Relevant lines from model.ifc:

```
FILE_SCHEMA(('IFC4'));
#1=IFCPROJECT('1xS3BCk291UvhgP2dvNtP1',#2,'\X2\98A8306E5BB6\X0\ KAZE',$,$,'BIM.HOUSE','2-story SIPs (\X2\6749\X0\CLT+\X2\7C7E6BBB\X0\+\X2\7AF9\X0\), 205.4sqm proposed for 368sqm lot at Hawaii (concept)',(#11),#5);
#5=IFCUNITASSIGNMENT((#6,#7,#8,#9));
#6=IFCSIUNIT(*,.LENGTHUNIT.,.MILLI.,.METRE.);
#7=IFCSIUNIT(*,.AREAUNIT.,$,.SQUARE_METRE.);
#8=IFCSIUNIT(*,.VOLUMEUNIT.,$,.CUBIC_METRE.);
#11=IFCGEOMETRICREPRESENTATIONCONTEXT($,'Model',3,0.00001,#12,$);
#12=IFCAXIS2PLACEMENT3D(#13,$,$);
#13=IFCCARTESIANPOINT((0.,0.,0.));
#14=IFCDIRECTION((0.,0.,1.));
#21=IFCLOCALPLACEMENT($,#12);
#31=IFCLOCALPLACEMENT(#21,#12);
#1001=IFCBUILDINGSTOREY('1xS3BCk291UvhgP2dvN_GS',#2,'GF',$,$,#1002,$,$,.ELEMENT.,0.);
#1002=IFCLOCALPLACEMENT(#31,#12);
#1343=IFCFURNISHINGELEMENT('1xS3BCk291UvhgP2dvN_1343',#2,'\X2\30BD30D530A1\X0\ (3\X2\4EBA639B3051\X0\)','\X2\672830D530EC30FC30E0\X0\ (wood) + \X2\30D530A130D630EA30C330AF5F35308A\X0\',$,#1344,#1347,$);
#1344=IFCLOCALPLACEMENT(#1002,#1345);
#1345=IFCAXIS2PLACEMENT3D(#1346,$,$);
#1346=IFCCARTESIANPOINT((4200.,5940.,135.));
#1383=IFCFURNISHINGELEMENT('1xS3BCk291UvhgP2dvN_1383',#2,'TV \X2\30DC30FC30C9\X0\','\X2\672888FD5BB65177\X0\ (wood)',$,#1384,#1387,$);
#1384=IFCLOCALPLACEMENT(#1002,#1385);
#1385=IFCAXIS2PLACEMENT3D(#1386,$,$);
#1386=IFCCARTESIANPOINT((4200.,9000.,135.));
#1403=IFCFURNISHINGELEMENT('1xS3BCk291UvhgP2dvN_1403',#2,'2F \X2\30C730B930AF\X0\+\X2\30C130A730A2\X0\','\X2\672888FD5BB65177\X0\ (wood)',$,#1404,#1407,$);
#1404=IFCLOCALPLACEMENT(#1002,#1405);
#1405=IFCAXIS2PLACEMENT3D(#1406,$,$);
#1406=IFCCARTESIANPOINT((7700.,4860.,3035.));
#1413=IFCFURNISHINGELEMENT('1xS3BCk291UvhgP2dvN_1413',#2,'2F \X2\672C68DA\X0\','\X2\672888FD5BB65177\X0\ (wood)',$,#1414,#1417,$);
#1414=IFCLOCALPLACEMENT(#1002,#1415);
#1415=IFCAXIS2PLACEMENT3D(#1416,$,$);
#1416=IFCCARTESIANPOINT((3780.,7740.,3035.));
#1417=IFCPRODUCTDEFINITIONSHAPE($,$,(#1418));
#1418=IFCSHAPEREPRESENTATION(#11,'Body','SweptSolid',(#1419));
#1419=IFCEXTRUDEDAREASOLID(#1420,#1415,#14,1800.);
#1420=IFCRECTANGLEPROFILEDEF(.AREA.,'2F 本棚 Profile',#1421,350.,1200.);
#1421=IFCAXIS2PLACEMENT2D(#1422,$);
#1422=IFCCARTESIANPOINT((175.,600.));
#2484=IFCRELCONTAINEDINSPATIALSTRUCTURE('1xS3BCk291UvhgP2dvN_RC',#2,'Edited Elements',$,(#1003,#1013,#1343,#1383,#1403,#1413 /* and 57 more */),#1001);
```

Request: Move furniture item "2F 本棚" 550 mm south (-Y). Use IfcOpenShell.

```python
import ifcopenshell
import ifcopenshell.api.geometry
import ifcopenshell.util.placement
import ifcopenshell.util.unit

model = ifcopenshell.open("model.ifc")
unit_scale = ifcopenshell.util.unit.calculate_unit_scale(model)

item = model.by_guid("1xS3BCk291UvhgP2dvN_1413")
matrix = ifcopenshell.util.placement.get_local_placement(item.ObjectPlacement)
matrix[1, 3] -= 0.55 / unit_scale
ifcopenshell.api.geometry.edit_object_placement(model, product=item, matrix=matrix, is_si=False)

print(ifcopenshell.util.placement.get_local_placement(item.ObjectPlacement).round(3) + 0.0)

model.write("model-out.ifc")
```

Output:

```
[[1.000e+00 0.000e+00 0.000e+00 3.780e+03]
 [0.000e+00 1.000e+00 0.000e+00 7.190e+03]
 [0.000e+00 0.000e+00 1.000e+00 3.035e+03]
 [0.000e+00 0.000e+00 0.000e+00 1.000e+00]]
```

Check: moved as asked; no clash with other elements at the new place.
